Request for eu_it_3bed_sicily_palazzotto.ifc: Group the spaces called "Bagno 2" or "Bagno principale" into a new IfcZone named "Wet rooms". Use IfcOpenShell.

First a look at what the model holds.

```python
import ifcopenshell

model = ifcopenshell.open("eu_it_3bed_sicily_palazzotto.ifc")
print(model.schema)
seen = {}
for space in model.by_type("IfcSpace"):
    seen[space.LongName] = seen.get(space.LongName, 0) + 1
for name, count in sorted(seen.items(), key=str):
    print(count, "x", name)
print("zones:", [z.Name for z in model.by_type("IfcZone")][:20])
```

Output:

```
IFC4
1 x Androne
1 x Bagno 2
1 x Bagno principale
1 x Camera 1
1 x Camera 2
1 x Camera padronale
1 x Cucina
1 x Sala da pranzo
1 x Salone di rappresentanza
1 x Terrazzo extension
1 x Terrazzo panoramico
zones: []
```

```python
import ifcopenshell
import ifcopenshell.api.group
import ifcopenshell.api.root

model = ifcopenshell.open("eu_it_3bed_sicily_palazzotto.ifc")

names = {"Bagno 2", "Bagno principale"}
spaces = [s for s in model.by_type("IfcSpace") if s.LongName in names]

zone = ifcopenshell.api.root.create_entity(model, ifc_class="IfcZone", name="Wet rooms")
ifcopenshell.api.group.assign_group(model, products=spaces, group=zone)
print(len(spaces), "spaces in", zone.Name)

model.write("eu_it_3bed_sicily_palazzotto_updated.ifc")
```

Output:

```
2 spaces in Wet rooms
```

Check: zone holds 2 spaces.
